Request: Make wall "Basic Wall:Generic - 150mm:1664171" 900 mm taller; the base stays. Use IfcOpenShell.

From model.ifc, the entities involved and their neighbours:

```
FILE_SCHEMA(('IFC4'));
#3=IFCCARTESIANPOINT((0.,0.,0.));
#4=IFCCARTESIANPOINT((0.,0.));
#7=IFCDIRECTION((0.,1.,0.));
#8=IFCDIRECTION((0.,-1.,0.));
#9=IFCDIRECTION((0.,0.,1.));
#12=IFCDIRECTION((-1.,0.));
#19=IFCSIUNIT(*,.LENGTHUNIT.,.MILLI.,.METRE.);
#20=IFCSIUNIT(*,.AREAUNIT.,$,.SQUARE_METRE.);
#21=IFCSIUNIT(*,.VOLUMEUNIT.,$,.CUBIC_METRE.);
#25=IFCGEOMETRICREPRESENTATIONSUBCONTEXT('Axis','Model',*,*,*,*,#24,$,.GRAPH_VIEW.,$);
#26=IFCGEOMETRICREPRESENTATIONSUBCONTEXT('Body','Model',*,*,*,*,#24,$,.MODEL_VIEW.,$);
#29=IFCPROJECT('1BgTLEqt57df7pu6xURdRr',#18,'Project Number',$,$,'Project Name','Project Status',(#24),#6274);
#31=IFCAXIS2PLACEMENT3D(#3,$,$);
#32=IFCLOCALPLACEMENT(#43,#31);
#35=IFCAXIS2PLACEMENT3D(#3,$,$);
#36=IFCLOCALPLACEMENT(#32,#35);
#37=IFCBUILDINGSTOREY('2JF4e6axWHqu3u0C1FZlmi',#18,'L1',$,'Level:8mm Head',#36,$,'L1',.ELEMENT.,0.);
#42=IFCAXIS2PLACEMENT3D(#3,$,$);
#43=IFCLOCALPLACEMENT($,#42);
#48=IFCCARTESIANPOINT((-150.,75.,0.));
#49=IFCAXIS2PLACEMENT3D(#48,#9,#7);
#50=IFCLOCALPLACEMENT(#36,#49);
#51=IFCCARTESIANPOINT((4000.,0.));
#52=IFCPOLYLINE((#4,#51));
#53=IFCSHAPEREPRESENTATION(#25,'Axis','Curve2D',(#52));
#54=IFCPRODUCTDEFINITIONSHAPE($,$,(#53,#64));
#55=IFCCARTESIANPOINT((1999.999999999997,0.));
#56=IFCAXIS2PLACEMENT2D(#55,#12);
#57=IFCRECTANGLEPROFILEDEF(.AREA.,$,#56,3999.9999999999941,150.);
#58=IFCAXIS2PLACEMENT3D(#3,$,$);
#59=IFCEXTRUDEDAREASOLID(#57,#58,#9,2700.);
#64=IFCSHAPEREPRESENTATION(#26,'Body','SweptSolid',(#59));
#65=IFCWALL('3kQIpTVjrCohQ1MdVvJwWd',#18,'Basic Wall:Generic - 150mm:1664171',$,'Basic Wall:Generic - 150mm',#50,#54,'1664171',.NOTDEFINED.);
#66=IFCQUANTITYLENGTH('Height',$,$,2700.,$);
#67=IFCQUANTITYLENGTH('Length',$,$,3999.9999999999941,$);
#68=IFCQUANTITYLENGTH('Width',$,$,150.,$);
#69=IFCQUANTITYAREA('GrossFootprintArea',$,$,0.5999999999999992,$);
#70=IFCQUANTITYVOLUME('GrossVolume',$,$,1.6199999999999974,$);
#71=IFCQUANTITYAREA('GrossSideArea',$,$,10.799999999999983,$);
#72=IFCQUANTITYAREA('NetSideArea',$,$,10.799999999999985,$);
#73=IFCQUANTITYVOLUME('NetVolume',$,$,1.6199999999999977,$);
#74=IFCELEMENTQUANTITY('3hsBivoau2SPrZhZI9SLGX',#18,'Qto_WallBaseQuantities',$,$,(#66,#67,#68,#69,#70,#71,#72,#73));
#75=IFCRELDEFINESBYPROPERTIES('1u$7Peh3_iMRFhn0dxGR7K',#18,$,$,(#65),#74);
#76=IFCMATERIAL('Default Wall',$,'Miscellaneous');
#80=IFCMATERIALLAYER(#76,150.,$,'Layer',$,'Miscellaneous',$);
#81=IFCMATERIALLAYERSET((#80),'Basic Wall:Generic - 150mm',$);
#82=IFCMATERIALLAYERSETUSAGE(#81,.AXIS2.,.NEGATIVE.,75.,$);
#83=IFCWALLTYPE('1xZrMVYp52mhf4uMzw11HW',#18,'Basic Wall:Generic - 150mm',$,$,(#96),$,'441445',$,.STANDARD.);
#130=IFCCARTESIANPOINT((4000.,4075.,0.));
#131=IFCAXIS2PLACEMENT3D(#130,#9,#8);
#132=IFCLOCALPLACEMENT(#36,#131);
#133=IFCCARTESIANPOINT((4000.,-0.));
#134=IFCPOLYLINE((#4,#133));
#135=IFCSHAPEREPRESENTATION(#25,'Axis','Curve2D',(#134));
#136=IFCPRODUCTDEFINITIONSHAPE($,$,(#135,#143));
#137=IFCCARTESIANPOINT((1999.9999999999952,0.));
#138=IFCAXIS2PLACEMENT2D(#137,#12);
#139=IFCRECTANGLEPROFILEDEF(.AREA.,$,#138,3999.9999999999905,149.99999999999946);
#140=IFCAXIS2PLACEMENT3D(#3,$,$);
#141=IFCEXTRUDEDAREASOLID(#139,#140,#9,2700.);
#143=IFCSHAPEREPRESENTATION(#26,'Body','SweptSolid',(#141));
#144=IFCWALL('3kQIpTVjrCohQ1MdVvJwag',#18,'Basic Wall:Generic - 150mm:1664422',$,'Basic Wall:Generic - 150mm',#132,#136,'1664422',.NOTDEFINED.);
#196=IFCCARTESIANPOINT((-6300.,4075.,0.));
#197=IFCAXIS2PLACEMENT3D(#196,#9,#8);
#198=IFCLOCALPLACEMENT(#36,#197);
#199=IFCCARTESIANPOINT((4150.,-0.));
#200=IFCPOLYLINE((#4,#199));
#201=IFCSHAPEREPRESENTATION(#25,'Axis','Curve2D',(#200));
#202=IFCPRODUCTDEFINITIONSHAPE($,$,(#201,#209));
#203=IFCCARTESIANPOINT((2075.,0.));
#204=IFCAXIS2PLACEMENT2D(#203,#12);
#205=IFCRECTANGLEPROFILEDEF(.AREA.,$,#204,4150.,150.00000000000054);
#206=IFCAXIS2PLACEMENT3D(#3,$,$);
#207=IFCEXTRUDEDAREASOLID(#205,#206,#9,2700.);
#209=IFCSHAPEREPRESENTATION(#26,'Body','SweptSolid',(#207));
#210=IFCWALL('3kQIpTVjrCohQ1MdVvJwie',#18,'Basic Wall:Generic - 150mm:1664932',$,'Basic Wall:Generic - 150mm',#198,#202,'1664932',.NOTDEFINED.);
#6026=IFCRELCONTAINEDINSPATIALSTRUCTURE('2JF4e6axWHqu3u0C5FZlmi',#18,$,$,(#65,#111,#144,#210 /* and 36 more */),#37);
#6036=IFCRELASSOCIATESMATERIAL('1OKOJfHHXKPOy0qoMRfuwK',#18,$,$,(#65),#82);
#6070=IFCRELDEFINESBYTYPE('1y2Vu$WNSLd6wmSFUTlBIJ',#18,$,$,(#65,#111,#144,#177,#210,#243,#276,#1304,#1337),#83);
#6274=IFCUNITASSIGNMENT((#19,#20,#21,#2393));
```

```python
import ifcopenshell
import ifcopenshell.api.pset
import ifcopenshell.geom
import ifcopenshell.util.element
import ifcopenshell.util.representation
import ifcopenshell.util.shape
import ifcopenshell.util.unit

model = ifcopenshell.open("model.ifc")
unit_scale = ifcopenshell.util.unit.calculate_unit_scale(model)
area_scale = ifcopenshell.util.unit.calculate_unit_scale(model, "AREAUNIT")
volume_scale = ifcopenshell.util.unit.calculate_unit_scale(model, "VOLUMEUNIT")
settings = ifcopenshell.geom.settings()


def volume(element):
    """Net volume in cubic metres, openings subtracted."""
    shape = ifcopenshell.geom.create_shape(settings, element)
    return ifcopenshell.util.shape.get_volume(shape.geometry)


wall = model.by_guid("3kQIpTVjrCohQ1MdVvJwWd")
before = volume(wall)

body = ifcopenshell.util.representation.get_representation(wall, "Model", "Body")
solid = body.Items[0]
old_height = solid.Depth
solid.Depth += 0.9 / unit_scale
after = volume(wall)
thickness = 0.15  # wall thickness in metres

# Update the stored height, areas and volumes.
qto = model.by_id(ifcopenshell.util.element.get_pset(wall, "Qto_WallBaseQuantities", should_inherit=False)["id"])
ifcopenshell.api.pset.edit_qto(model, qto=qto, properties={
    "Height": solid.Depth,
    "GrossVolume": ifcopenshell.util.element.get_pset(wall, "Qto_WallBaseQuantities", "GrossVolume") * solid.Depth / old_height,
    "GrossSideArea": ifcopenshell.util.element.get_pset(wall, "Qto_WallBaseQuantities", "GrossSideArea") * solid.Depth / old_height,
    "NetSideArea": after / thickness / area_scale,
    "NetVolume": after / volume_scale,
})

print(f"height {old_height:g} -> {solid.Depth:g}, volume {before:.3f} -> {after:.3f} m3")

model.write("model_edited.ifc")
```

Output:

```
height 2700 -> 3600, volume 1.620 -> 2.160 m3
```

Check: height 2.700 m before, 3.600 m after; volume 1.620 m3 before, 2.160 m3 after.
